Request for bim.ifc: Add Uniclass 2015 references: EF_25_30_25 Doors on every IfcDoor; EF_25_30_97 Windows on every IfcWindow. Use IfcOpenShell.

First a look at what the model holds.

```python
import ifcopenshell

model = ifcopenshell.open("bim.ifc")
print(model.schema)
print("classifications:", [c.Name for c in model.by_type("IfcClassification")])
for ifc_class in ("IfcDoor", "IfcRoof", "IfcStair", "IfcWall", "IfcWindow"):
    print(ifc_class, len(model.by_type(ifc_class)))
```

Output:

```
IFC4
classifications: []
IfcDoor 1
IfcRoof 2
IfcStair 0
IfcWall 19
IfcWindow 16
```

```python
import ifcopenshell
import ifcopenshell.api.classification

model = ifcopenshell.open("bim.ifc")

system = ifcopenshell.api.classification.add_classification(model, classification="Uniclass 2015")

codes = {
    "IfcDoor": ("EF_25_30_25", "Doors"),
    "IfcWindow": ("EF_25_30_97", "Windows"),
}
for ifc_class, (code, name) in codes.items():
    products = model.by_type(ifc_class)
    ifcopenshell.api.classification.add_reference(
        model, products=products, classification=system, identification=code, name=name
    )
    print(code, len(products))

model.write("bim_edited.ifc")
```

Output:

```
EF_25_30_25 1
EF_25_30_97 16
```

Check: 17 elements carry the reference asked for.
